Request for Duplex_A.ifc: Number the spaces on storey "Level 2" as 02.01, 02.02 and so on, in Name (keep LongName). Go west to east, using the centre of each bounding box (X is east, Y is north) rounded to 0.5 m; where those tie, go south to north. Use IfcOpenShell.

First a look at what the model holds.

```python
import ifcopenshell
import ifcopenshell.util.element
import ifcopenshell.util.placement

model = ifcopenshell.open("Duplex_A.ifc")
print(model.schema)
storey = next(s for s in model.by_type("IfcBuildingStorey") if s.Name == "Level 2")
spaces = [e for e in ifcopenshell.util.element.get_decomposition(storey) if e.is_a("IfcSpace")]
for e in sorted(spaces, key=lambda e: e.id()):
    origin = ifcopenshell.util.placement.get_local_placement(e.ObjectPlacement)[:3, 3]
    print(e.id(), e.Name, e.LongName, origin.round(2) + 0.0, sep=" | ")
```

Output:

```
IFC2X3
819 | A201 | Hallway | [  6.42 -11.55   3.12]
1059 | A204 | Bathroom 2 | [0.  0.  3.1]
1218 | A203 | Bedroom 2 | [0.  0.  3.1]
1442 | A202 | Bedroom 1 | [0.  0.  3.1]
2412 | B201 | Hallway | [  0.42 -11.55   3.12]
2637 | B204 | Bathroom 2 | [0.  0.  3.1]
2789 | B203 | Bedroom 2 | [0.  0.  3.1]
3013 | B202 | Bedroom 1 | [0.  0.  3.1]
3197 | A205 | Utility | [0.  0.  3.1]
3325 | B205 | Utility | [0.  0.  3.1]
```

```python
import ifcopenshell
import ifcopenshell.geom
import ifcopenshell.util.element
import ifcopenshell.util.shape

model = ifcopenshell.open("Duplex_A.ifc")
settings = ifcopenshell.geom.settings()
settings.set("use-world-coords", True)


def centre(element):
    shape = ifcopenshell.geom.create_shape(settings, element)
    return ifcopenshell.util.shape.get_bbox_centroid(shape.geometry)


storey = next(s for s in model.by_type("IfcBuildingStorey") if s.Name == "Level 2")
spaces = [e for e in ifcopenshell.util.element.get_decomposition(storey) if e.is_a("IfcSpace")]

# Insertion points can sit at a corner or the storey origin, so sort by the geometry (in metres).
centres = {e: centre(e) for e in spaces}
spaces.sort(key=lambda e: (round(centres[e][0] / 0.5), centres[e][1]))

for i, e in enumerate(spaces, start=1):
    number = f"02.{i:02d}"
    e.Name = number
    print(e.id(), number)

model.write("Duplex_A-out.ifc")
```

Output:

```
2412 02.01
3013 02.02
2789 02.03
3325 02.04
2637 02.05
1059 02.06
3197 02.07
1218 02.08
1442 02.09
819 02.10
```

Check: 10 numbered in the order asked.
